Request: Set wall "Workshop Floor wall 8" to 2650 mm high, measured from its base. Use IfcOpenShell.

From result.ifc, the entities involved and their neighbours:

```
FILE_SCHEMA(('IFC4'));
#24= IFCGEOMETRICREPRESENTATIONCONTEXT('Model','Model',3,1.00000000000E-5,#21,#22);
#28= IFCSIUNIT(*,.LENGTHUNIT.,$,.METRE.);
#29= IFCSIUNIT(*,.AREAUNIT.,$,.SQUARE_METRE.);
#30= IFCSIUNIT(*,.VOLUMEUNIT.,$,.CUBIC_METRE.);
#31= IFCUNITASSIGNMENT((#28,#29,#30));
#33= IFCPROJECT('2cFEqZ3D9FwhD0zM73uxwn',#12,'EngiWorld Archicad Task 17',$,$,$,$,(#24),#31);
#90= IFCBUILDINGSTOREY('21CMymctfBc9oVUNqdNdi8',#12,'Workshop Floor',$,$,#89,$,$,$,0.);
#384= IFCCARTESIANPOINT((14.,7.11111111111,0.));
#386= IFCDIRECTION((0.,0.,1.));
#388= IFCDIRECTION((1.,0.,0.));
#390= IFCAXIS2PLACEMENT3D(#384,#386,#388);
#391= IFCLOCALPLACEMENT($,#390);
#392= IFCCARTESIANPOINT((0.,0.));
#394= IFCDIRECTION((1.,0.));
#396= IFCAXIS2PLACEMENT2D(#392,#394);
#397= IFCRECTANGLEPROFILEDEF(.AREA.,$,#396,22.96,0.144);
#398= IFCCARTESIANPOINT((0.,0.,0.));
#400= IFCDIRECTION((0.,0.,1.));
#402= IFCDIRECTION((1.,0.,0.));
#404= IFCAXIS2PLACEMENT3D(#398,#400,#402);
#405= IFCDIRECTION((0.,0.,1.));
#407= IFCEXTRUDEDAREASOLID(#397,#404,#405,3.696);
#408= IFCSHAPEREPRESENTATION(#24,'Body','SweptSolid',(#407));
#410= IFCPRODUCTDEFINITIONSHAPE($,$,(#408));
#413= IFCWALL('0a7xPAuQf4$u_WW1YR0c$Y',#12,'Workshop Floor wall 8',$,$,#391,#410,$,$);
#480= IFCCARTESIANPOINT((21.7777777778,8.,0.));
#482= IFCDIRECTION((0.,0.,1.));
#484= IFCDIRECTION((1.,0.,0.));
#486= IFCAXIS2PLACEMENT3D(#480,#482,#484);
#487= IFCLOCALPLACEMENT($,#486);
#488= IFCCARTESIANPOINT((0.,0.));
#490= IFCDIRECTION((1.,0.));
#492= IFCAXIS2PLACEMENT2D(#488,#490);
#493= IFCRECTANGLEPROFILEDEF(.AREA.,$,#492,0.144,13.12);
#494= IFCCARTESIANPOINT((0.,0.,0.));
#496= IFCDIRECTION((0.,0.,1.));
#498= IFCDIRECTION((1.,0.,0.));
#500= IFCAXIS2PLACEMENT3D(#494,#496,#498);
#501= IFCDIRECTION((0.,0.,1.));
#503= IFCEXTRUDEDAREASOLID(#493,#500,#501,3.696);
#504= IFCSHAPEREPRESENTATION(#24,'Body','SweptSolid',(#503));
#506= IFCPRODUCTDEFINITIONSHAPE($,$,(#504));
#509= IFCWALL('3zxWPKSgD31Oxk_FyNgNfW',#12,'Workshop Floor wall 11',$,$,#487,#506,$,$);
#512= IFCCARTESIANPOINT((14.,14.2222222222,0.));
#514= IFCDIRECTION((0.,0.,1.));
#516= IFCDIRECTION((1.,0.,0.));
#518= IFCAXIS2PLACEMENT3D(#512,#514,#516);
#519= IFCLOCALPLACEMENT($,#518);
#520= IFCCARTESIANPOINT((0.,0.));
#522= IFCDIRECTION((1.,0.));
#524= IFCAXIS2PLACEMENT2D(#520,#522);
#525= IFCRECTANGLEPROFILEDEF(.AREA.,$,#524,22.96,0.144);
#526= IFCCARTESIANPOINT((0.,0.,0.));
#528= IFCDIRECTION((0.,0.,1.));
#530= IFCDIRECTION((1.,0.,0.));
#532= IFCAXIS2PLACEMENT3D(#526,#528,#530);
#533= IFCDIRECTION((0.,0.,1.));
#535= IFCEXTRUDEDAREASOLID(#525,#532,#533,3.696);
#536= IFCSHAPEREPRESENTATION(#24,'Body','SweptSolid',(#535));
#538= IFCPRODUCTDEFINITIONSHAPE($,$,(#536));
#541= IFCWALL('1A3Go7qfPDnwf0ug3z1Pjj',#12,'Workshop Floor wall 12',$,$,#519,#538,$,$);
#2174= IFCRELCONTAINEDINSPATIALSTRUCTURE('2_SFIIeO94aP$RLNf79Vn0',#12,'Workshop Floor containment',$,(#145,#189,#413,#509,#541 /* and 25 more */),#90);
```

```python
import ifcopenshell
import ifcopenshell.geom
import ifcopenshell.util.shape

model = ifcopenshell.open("result.ifc")
settings = ifcopenshell.geom.settings()


def volume(element):
    """Net volume in cubic metres, openings subtracted."""
    shape = ifcopenshell.geom.create_shape(settings, element)
    return ifcopenshell.util.shape.get_volume(shape.geometry)


wall = model.by_guid("0a7xPAuQf4$u_WW1YR0c$Y")
before = volume(wall)

body = next(r for r in wall.Representation.Representations if r.RepresentationIdentifier == "Body")
solid = body.Items[0]
old_height = solid.Depth
solid.Depth = 2.65
after = volume(wall)

print(f"height {old_height:g} -> {solid.Depth:g}, volume {before:.3f} -> {after:.3f} m3")

model.write("result-out.ifc")
```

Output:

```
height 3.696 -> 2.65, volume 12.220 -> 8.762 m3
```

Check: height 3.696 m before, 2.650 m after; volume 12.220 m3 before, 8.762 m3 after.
